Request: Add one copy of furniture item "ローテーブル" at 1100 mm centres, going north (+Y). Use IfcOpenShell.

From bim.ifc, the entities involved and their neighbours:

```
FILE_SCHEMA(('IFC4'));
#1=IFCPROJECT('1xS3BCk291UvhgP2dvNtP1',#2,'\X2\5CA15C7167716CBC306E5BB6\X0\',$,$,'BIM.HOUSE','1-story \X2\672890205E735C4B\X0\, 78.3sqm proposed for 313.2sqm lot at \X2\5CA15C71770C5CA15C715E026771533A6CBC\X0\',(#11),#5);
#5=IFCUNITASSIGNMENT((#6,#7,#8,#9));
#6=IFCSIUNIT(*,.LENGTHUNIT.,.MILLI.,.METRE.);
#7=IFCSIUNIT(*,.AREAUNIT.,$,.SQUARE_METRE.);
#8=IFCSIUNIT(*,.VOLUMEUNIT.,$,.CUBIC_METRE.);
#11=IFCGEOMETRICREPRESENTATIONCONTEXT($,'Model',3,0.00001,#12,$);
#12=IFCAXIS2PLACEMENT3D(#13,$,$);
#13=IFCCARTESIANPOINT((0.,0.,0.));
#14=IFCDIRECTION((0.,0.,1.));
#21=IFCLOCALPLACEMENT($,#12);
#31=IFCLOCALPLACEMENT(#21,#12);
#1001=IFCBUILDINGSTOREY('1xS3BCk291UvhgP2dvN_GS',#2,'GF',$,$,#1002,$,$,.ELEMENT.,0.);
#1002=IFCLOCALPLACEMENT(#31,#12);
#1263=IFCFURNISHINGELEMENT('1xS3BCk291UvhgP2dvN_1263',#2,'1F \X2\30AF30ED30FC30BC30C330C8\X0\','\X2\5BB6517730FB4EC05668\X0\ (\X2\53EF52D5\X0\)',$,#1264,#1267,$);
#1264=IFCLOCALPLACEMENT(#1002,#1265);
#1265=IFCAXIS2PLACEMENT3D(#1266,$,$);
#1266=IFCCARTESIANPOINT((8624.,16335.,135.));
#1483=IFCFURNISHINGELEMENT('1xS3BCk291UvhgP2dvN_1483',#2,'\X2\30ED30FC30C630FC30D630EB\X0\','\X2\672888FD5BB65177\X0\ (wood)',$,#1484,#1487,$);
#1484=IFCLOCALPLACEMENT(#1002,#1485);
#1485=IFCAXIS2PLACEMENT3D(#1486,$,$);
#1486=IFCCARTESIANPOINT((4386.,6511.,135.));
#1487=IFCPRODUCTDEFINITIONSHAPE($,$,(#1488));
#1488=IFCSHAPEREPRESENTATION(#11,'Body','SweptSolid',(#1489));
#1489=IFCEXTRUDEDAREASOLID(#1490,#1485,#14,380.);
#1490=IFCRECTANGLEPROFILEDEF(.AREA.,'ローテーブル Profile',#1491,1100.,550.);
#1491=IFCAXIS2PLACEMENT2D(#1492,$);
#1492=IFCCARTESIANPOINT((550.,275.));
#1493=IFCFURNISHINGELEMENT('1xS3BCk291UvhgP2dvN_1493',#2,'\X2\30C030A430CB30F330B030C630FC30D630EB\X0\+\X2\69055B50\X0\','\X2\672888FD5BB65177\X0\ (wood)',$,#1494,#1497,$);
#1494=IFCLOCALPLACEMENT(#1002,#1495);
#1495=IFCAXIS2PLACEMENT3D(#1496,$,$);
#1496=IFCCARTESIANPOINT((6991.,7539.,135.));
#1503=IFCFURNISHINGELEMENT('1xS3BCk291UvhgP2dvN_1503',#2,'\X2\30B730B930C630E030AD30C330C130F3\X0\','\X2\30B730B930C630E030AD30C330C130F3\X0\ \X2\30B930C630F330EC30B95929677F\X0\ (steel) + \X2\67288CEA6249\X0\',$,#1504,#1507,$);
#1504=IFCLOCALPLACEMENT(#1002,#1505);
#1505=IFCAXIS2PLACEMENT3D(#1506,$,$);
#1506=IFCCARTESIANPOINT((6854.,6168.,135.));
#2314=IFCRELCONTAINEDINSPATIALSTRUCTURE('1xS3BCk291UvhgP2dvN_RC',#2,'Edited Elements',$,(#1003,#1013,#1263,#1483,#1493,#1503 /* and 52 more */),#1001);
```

```python
import numpy as np
import ifcopenshell
import ifcopenshell.api.geometry
import ifcopenshell.api.root
import ifcopenshell.util.element
import ifcopenshell.util.placement

model = ifcopenshell.open("bim.ifc")


def reuse_history(source, copy):
    """copy_class also copies each property set's owner history, people and application; keep the originals."""
    for rel in copy.IsDefinedBy:
        if rel.is_a("IfcRelDefinesByProperties") and (history := rel.RelatingPropertyDefinition.OwnerHistory):
            rel.RelatingPropertyDefinition.OwnerHistory = source.OwnerHistory
            ifcopenshell.util.element.remove_deep2(model, history)


source = model.by_guid("1xS3BCk291UvhgP2dvN_1483")
base = ifcopenshell.util.placement.get_local_placement(source.ObjectPlacement)
step = np.array([0.0, 1.0, 0.0]) * 1100.0

for i in range(1, 2):
    copy = ifcopenshell.api.root.copy_class(model, product=source)
    copy.Representation = ifcopenshell.util.element.copy_deep(
        model, source.Representation, exclude=["IfcGeometricRepresentationContext", "IfcRepresentationMap"]
    )
    reuse_history(source, copy)
    matrix = base.copy()
    matrix[:3, 3] += i * step
    print("added at", matrix[:3, 3].round(3) + 0.0)
    ifcopenshell.api.geometry.edit_object_placement(model, product=copy, matrix=matrix, is_si=False)

model.write("bim_rev.ifc")
```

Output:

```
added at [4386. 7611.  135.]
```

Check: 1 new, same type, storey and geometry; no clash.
